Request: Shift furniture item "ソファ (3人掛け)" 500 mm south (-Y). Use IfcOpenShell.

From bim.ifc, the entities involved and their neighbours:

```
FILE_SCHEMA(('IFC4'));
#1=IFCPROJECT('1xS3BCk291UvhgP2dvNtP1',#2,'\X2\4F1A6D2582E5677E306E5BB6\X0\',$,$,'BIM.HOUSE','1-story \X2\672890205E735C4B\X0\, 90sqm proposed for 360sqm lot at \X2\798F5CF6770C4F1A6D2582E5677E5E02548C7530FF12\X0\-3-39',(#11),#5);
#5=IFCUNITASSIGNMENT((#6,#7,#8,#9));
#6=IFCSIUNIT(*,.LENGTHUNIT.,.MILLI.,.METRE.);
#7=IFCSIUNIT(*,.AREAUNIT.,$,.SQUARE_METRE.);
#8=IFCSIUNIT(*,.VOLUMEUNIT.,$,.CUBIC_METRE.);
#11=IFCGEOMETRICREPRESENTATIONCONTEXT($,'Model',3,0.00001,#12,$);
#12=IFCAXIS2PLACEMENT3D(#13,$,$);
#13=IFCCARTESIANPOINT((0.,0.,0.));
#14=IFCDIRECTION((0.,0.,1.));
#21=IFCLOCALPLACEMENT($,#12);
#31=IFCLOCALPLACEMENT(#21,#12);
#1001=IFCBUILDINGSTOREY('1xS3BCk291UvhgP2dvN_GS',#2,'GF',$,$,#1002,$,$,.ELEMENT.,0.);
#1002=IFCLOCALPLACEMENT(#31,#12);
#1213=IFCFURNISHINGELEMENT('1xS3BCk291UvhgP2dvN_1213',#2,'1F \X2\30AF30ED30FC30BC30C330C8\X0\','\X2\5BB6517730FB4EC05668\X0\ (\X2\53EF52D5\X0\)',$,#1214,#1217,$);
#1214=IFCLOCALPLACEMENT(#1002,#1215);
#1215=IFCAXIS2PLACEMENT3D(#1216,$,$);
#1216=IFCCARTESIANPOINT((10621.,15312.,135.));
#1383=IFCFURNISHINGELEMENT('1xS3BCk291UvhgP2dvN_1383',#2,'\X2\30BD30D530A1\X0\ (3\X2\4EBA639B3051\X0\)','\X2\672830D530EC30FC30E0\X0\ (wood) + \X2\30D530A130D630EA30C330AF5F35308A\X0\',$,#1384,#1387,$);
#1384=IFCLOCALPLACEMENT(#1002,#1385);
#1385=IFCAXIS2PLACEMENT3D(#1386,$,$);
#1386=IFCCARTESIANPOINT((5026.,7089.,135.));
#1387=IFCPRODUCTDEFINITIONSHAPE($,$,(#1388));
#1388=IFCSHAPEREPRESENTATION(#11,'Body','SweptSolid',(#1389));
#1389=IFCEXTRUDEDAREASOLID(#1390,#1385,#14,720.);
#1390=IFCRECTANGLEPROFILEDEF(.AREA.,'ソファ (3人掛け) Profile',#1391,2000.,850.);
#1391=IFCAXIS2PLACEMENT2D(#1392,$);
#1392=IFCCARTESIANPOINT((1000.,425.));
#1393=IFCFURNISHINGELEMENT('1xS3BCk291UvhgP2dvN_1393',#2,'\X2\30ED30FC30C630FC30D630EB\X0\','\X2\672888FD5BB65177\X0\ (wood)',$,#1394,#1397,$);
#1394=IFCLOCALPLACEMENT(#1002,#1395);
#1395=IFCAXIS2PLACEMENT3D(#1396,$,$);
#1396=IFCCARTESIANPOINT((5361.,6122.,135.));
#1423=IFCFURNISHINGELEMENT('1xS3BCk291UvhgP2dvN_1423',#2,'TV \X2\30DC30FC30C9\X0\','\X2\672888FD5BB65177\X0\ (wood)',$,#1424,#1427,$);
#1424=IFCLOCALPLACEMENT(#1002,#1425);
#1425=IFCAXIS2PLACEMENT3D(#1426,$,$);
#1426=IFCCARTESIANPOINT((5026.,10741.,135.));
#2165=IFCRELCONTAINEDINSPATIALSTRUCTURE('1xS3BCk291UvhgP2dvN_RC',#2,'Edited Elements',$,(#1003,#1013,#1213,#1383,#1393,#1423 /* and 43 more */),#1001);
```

```python
import ifcopenshell
import ifcopenshell.api.geometry
import ifcopenshell.util.placement
import ifcopenshell.util.unit

model = ifcopenshell.open("bim.ifc")
unit_scale = ifcopenshell.util.unit.calculate_unit_scale(model)

item = model.by_guid("1xS3BCk291UvhgP2dvN_1383")
matrix = ifcopenshell.util.placement.get_local_placement(item.ObjectPlacement)
matrix[1, 3] -= 0.5 / unit_scale
ifcopenshell.api.geometry.edit_object_placement(model, product=item, matrix=matrix, is_si=False)

print(ifcopenshell.util.placement.get_local_placement(item.ObjectPlacement).round(3) + 0.0)

model.write("bim_v2.ifc")
```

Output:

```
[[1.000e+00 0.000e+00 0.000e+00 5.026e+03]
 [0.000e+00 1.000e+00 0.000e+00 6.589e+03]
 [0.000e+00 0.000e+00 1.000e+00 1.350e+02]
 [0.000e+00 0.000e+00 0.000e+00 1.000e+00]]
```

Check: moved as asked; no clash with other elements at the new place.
